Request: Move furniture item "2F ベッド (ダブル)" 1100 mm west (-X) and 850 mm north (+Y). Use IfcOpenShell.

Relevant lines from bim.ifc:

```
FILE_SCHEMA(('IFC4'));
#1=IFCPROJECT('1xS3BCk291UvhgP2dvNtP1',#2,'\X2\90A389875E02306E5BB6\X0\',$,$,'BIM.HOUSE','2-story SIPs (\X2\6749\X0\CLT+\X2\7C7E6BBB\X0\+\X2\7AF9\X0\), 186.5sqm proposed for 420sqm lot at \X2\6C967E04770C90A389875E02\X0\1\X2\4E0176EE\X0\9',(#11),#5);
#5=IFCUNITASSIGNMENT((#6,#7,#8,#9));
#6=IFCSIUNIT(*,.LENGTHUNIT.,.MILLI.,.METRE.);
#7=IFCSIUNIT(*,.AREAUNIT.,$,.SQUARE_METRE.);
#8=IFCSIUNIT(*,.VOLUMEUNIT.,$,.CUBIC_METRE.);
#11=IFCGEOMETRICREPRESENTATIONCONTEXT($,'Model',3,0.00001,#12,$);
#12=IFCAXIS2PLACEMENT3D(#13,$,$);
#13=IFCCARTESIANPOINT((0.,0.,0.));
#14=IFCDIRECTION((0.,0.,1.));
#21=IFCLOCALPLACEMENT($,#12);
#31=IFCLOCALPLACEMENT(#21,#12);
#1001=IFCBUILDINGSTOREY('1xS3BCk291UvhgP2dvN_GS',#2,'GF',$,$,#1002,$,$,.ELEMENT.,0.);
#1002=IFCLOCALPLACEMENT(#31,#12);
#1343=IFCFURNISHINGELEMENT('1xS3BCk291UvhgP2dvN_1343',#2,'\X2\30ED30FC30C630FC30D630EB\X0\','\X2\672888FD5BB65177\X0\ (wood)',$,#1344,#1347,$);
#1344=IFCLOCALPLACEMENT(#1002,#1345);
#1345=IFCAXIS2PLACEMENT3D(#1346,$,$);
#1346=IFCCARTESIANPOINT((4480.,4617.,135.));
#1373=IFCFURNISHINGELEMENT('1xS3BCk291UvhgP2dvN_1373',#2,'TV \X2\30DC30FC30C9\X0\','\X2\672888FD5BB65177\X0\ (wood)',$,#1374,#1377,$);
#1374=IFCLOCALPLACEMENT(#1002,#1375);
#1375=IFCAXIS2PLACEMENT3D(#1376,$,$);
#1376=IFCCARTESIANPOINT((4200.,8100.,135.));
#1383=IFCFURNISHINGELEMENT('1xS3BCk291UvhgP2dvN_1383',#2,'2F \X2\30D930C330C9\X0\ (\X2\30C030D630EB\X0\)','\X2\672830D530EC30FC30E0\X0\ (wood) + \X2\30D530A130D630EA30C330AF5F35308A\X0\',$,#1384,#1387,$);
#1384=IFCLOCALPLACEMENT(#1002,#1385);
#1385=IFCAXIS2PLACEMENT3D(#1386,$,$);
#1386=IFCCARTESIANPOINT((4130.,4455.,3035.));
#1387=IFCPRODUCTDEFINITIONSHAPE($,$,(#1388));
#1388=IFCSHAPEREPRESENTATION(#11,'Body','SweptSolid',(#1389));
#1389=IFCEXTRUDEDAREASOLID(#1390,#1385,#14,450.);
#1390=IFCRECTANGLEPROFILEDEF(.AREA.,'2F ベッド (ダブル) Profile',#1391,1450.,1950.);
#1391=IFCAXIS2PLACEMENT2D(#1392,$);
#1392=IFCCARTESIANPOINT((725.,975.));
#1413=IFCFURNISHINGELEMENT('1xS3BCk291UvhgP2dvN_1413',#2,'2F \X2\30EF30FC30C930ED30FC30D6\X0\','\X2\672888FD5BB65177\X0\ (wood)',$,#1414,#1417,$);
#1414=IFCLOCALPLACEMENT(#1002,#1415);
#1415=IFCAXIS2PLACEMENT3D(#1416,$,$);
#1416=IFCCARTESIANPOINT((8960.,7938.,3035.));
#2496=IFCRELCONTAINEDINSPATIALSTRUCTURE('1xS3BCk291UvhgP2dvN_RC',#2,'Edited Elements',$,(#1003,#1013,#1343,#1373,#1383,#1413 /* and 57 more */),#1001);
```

```python
import ifcopenshell
import ifcopenshell.api.geometry
import ifcopenshell.util.placement
import ifcopenshell.util.unit

model = ifcopenshell.open("bim.ifc")
unit_scale = ifcopenshell.util.unit.calculate_unit_scale(model)

item = model.by_guid("1xS3BCk291UvhgP2dvN_1383")
matrix = ifcopenshell.util.placement.get_local_placement(item.ObjectPlacement)
matrix[0, 3] -= 1.1 / unit_scale
matrix[1, 3] += 0.85 / unit_scale
ifcopenshell.api.geometry.edit_object_placement(model, product=item, matrix=matrix, is_si=False)

print(ifcopenshell.util.placement.get_local_placement(item.ObjectPlacement).round(3) + 0.0)

model.write("bim-out.ifc")
```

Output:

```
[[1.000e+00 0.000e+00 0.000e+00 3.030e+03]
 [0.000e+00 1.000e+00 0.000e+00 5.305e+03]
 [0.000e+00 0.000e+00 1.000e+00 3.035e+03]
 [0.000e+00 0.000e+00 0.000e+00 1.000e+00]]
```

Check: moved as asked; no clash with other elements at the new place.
